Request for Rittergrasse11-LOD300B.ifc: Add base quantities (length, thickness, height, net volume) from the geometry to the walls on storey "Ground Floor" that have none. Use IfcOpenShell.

First a look at what the model holds.

```python
import ifcopenshell
import ifcopenshell.util.element
import ifcopenshell.util.unit

model = ifcopenshell.open("Rittergrasse11-LOD300B.ifc")
print(model.schema)
for unit_type in ("LENGTHUNIT", "AREAUNIT", "VOLUMEUNIT"):
    print(unit_type, ifcopenshell.util.unit.calculate_unit_scale(model, unit_type))
storey = next(s for s in model.by_type("IfcBuildingStorey") if s.Name == "Ground Floor")
walls = [e for e in ifcopenshell.util.element.get_decomposition(storey) if e.is_a("IfcWall")]
for e in sorted(walls, key=lambda e: e.id()):
    print(e.id(), e.is_a(), e.Name, list(ifcopenshell.util.element.get_psets(e, qtos_only=True)), sep=" | ")
```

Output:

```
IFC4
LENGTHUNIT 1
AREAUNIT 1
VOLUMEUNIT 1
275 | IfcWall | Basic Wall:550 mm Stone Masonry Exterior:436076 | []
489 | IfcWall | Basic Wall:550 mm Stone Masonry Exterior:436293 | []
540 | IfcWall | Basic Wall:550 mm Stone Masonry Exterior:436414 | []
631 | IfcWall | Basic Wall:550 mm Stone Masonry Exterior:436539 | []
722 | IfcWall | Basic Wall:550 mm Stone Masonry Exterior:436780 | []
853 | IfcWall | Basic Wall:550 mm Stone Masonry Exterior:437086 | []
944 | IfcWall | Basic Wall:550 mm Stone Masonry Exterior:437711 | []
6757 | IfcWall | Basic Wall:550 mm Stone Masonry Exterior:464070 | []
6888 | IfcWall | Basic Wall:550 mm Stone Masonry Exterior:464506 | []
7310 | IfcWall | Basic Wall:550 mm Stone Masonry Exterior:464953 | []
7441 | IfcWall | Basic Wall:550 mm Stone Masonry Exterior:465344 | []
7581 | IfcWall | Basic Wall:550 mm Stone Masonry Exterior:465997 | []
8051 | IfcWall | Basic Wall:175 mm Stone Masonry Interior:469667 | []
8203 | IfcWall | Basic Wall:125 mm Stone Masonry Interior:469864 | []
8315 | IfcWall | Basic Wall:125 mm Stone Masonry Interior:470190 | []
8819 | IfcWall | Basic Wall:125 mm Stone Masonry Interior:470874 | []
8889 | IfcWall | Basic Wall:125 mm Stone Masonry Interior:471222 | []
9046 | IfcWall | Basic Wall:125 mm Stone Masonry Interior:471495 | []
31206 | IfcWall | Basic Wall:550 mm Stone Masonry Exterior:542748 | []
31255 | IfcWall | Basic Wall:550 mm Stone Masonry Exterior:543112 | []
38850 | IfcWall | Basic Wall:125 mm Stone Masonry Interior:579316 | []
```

```python
import ifcopenshell
import ifcopenshell.api.pset
import ifcopenshell.geom
import ifcopenshell.util.element
import ifcopenshell.util.shape
import ifcopenshell.util.unit

model = ifcopenshell.open("Rittergrasse11-LOD300B.ifc")
unit_scale = ifcopenshell.util.unit.calculate_unit_scale(model)
volume_scale = ifcopenshell.util.unit.calculate_unit_scale(model, "VOLUMEUNIT")
settings = ifcopenshell.geom.settings()

storey = next(s for s in model.by_type("IfcBuildingStorey") if s.Name == "Ground Floor")
walls = [e for e in ifcopenshell.util.element.get_decomposition(storey) if e.is_a("IfcWall")]

for e in sorted(walls, key=lambda e: e.id()):
    if ifcopenshell.util.element.get_psets(e, qtos_only=True, should_inherit=False):
        continue
    # Geometry comes back in metres, in the element's own axes.
    shape = ifcopenshell.geom.create_shape(settings, e)
    values = {
        "Length": ifcopenshell.util.shape.get_x(shape.geometry) / unit_scale,
        "Width": ifcopenshell.util.shape.get_y(shape.geometry) / unit_scale,
        "Height": ifcopenshell.util.shape.get_z(shape.geometry) / unit_scale,
        "NetVolume": ifcopenshell.util.shape.get_volume(shape.geometry) / volume_scale,
    }
    qto = ifcopenshell.api.pset.add_qto(model, product=e, name="Qto_WallBaseQuantities")
    ifcopenshell.api.pset.edit_qto(model, qto=qto, properties=values)
    print(e.id(), {k: round(v, 3) for k, v in values.items()})

model.write("Rittergrasse11-LOD300B_rev.ifc")
```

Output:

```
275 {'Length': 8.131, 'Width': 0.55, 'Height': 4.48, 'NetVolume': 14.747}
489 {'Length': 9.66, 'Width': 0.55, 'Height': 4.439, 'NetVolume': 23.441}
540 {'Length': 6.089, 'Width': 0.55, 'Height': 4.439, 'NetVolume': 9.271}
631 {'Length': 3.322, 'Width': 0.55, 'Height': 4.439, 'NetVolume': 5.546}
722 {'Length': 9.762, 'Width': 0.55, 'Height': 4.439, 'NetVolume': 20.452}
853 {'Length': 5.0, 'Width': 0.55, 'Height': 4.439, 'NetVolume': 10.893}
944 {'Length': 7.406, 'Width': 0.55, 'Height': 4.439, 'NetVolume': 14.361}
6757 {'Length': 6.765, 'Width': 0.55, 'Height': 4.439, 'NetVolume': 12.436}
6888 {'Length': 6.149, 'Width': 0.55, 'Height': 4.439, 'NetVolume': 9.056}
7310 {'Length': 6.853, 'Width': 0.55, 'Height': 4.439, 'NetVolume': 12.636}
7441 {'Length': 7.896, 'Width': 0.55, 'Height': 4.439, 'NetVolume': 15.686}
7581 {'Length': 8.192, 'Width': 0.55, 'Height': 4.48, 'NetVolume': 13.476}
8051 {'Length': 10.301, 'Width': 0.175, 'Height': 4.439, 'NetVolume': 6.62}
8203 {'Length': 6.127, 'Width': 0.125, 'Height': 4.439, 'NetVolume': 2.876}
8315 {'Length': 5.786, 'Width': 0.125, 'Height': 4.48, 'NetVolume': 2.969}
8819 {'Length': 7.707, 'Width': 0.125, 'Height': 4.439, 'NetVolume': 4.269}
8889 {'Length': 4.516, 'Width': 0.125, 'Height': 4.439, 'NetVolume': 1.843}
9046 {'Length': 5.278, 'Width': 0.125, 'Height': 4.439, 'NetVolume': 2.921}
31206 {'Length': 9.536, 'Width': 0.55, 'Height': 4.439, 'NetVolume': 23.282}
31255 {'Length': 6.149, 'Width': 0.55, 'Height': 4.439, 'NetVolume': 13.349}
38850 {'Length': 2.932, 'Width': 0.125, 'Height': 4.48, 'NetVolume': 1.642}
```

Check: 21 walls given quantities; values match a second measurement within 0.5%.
